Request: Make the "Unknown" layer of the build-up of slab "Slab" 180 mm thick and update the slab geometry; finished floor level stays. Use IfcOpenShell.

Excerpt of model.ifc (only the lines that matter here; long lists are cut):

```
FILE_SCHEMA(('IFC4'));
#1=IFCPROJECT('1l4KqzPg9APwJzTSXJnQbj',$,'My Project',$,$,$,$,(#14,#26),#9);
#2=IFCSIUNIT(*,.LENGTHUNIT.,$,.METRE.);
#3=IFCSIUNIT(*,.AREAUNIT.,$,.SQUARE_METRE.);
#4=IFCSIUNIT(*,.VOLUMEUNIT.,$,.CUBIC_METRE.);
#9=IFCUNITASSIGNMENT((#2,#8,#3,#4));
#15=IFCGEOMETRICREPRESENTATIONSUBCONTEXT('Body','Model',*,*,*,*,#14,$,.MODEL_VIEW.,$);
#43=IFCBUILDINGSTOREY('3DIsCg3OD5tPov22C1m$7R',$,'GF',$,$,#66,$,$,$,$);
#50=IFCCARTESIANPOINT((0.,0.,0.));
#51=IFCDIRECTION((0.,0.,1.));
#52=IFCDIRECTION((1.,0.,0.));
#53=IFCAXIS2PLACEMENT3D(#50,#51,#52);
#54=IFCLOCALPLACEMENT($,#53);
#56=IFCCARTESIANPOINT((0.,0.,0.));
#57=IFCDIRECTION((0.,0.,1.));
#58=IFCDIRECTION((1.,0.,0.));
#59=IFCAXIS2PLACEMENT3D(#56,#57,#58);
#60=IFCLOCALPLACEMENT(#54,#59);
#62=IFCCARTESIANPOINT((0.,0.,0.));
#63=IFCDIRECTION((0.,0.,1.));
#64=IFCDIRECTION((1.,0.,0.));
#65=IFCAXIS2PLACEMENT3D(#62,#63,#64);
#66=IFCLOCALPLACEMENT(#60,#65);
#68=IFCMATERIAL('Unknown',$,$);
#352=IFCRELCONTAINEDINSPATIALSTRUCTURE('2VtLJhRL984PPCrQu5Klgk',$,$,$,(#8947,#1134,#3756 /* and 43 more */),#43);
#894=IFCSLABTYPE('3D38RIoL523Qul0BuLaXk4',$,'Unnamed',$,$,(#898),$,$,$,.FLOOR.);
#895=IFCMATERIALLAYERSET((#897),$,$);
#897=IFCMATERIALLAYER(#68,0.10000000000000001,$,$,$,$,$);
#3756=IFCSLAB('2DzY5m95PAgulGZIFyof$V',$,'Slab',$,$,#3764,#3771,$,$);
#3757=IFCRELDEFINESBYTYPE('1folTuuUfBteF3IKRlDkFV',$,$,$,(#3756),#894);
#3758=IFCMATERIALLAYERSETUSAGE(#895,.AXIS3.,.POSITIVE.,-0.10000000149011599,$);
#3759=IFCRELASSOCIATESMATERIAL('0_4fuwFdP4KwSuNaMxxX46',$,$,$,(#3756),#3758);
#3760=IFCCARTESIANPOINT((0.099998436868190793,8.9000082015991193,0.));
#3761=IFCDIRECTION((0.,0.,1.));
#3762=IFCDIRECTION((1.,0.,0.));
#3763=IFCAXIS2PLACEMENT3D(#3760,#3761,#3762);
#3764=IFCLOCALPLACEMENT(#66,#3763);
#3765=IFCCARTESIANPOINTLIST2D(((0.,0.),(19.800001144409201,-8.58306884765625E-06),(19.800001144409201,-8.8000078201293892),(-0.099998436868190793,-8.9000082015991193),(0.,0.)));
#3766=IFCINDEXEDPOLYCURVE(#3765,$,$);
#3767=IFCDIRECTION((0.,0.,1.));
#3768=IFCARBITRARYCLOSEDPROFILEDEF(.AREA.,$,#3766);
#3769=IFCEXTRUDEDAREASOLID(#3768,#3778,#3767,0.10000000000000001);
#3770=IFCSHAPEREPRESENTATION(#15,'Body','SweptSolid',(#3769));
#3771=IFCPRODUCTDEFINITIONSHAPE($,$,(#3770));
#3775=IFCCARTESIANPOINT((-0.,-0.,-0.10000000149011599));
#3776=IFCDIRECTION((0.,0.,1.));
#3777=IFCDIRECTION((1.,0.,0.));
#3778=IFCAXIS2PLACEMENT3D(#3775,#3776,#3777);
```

```python
import ifcopenshell
import ifcopenshell.util.element
import ifcopenshell.util.representation
import ifcopenshell.util.unit

model = ifcopenshell.open("model.ifc")
unit_scale = ifcopenshell.util.unit.calculate_unit_scale(model)

layer_set = model.by_id(895)
layer = next(l for l in layer_set.MaterialLayers if l.Material and l.Material.Name == "Unknown")
change = 0.18 / unit_scale - layer.LayerThickness
layer.LayerThickness += change

# Geometry does not follow the layer set by itself.
slabs = [e for e in ifcopenshell.util.element.get_elements_by_material(model, layer_set) if e.is_a("IfcSlab")]
for slab in sorted(slabs, key=lambda e: e.id()):
    body = ifcopenshell.util.representation.get_representation(slab, "Model", "Body")
    solid = body.Items[0]
    old_depth = solid.Depth
    solid.Depth += change
    # Extruded upwards: lower the start of the extrusion so the top stays.
    x, y, z = solid.Position.Location.Coordinates
    solid.Position.Location = model.createIfcCartesianPoint((x, y, z - change))
    print(slab.id(), f"{old_depth:g} -> {solid.Depth:g}")

# The layers are counted up from the underside, which has moved.
for usage in {ifcopenshell.util.element.get_material(slab) for slab in slabs}:
    usage.OffsetFromReferenceLine -= change

model.write("model_v2.ifc")
```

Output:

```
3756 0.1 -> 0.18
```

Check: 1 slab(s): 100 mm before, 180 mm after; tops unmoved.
